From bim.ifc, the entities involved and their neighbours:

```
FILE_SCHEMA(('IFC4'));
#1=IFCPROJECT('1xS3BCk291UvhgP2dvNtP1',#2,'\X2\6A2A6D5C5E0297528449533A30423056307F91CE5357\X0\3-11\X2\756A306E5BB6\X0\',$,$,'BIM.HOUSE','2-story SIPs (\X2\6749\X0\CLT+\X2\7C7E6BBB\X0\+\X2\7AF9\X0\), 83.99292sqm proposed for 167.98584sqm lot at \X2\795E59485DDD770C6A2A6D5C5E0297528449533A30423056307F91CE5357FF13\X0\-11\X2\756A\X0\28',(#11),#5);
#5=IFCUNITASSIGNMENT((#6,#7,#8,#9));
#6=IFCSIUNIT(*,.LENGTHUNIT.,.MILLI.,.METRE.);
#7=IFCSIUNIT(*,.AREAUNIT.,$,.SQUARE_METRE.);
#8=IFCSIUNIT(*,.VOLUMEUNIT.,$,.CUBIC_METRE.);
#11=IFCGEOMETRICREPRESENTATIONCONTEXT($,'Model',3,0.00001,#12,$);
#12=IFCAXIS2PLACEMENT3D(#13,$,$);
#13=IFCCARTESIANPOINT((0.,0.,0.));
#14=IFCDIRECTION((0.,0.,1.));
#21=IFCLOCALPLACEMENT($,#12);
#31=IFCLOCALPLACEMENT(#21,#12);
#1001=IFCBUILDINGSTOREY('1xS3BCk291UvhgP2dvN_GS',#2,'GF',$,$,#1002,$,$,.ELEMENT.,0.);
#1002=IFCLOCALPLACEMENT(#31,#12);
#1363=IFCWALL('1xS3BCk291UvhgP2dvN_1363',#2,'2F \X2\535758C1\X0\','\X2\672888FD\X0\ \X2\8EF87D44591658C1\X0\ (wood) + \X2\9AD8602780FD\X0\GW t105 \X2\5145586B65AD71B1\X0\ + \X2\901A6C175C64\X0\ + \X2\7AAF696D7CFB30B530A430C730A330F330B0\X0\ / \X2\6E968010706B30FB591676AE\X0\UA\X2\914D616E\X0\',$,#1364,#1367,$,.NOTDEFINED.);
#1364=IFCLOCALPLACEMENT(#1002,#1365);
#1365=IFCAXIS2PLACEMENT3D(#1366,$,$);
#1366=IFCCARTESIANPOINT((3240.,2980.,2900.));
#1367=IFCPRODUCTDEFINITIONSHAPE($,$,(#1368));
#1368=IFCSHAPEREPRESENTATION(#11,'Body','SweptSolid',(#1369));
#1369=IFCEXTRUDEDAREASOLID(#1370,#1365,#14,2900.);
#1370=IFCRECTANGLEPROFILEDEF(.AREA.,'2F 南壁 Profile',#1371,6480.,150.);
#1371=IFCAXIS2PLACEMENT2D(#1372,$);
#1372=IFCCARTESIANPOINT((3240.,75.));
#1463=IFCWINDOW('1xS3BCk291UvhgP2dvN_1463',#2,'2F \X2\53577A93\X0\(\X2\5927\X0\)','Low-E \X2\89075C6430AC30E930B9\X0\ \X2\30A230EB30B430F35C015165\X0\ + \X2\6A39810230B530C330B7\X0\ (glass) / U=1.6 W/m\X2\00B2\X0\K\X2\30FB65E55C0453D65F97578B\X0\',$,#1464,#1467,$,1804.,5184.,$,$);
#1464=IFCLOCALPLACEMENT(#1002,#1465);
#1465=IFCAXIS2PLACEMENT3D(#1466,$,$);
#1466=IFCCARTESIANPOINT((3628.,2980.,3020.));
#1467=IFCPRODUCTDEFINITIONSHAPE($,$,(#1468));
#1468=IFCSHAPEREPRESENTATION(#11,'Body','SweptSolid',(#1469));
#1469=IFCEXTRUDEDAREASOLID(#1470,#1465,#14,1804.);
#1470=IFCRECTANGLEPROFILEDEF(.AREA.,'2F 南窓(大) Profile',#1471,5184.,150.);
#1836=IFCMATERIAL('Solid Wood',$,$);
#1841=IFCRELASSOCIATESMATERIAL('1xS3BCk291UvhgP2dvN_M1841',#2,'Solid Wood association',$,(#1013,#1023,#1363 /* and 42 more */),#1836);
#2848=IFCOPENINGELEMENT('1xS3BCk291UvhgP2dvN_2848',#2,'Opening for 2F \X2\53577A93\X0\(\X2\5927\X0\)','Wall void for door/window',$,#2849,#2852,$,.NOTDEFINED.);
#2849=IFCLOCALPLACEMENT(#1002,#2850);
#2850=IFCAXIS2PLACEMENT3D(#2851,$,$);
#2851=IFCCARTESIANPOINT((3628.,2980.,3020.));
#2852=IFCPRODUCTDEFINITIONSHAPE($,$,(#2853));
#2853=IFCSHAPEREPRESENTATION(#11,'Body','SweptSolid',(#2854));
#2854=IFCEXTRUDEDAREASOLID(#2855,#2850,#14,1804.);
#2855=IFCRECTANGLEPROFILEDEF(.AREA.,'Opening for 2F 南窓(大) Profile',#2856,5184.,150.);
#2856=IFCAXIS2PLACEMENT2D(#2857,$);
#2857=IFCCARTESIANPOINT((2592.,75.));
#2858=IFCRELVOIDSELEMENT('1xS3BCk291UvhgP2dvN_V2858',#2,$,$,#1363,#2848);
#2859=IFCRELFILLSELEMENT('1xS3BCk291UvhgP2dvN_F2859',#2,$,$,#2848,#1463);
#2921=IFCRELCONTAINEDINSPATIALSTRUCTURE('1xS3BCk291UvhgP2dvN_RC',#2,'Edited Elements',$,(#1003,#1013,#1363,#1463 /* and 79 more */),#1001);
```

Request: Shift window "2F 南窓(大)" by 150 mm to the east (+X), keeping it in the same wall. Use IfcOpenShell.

```python
import ifcopenshell
import ifcopenshell.api.geometry
import ifcopenshell.util.placement

model = ifcopenshell.open("bim.ifc")

window = model.by_guid("1xS3BCk291UvhgP2dvN_1463")
opening = window.FillsVoids[0].RelatingOpeningElement
wall = opening.VoidsElements[0].RelatingBuildingElement

wall_matrix = ifcopenshell.util.placement.get_local_placement(wall.ObjectPlacement)
shift = wall_matrix[:3, 0] * 150.0
before = ifcopenshell.util.placement.get_local_placement(window.ObjectPlacement)[:3, 3].copy()

# The window is not placed relative to its opening, so move both.
for product in (opening, window):
    matrix = ifcopenshell.util.placement.get_local_placement(product.ObjectPlacement)
    matrix[:3, 3] += shift
    ifcopenshell.api.geometry.edit_object_placement(model, product=product, matrix=matrix, is_si=False)

after = ifcopenshell.util.placement.get_local_placement(window.ObjectPlacement)[:3, 3]
print("window moved by", (after - before).round(3) + 0.0)

model.write("bim_v2.ifc")
```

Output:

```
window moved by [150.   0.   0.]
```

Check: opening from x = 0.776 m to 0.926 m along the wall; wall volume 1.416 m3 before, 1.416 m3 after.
